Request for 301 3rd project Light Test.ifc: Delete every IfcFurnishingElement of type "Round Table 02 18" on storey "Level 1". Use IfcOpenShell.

First a look at what the model holds.

```python
import ifcopenshell
import ifcopenshell.util.element

model = ifcopenshell.open("301 3rd project Light Test.ifc")
print(model.schema)
storey = next(s for s in model.by_type("IfcBuildingStorey") if s.Name == "Level 1")
furniture = [e for e in ifcopenshell.util.element.get_decomposition(storey) if e.is_a("IfcFurnishingElement")]
seen = {}
for e in furniture:
    element_type = ifcopenshell.util.element.get_type(e)
    name = element_type.Name if element_type not in (None, e) else None
    seen[name] = seen.get(name, 0) + 1
for name, count in sorted(seen.items(), key=str):
    print(count, "x", name)
```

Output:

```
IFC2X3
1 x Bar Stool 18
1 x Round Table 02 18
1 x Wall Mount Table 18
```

```python
import ifcopenshell
import ifcopenshell.api.root
import ifcopenshell.util.element

model = ifcopenshell.open("301 3rd project Light Test.ifc")

storey = next(s for s in model.by_type("IfcBuildingStorey") if s.Name == "Level 1")
furniture = [e for e in ifcopenshell.util.element.get_decomposition(storey) if e.is_a("IfcFurnishingElement")]
targets = [e for e in furniture if (t := ifcopenshell.util.element.get_type(e)) not in (None, e) and t.Name == "Round Table 02 18"]

for e in targets:
    ifcopenshell.api.root.remove_product(model, product=e)
print(len(targets), "removed")

model.write("301 3rd project Light Test_rev.ifc")
```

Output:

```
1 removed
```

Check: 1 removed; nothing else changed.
